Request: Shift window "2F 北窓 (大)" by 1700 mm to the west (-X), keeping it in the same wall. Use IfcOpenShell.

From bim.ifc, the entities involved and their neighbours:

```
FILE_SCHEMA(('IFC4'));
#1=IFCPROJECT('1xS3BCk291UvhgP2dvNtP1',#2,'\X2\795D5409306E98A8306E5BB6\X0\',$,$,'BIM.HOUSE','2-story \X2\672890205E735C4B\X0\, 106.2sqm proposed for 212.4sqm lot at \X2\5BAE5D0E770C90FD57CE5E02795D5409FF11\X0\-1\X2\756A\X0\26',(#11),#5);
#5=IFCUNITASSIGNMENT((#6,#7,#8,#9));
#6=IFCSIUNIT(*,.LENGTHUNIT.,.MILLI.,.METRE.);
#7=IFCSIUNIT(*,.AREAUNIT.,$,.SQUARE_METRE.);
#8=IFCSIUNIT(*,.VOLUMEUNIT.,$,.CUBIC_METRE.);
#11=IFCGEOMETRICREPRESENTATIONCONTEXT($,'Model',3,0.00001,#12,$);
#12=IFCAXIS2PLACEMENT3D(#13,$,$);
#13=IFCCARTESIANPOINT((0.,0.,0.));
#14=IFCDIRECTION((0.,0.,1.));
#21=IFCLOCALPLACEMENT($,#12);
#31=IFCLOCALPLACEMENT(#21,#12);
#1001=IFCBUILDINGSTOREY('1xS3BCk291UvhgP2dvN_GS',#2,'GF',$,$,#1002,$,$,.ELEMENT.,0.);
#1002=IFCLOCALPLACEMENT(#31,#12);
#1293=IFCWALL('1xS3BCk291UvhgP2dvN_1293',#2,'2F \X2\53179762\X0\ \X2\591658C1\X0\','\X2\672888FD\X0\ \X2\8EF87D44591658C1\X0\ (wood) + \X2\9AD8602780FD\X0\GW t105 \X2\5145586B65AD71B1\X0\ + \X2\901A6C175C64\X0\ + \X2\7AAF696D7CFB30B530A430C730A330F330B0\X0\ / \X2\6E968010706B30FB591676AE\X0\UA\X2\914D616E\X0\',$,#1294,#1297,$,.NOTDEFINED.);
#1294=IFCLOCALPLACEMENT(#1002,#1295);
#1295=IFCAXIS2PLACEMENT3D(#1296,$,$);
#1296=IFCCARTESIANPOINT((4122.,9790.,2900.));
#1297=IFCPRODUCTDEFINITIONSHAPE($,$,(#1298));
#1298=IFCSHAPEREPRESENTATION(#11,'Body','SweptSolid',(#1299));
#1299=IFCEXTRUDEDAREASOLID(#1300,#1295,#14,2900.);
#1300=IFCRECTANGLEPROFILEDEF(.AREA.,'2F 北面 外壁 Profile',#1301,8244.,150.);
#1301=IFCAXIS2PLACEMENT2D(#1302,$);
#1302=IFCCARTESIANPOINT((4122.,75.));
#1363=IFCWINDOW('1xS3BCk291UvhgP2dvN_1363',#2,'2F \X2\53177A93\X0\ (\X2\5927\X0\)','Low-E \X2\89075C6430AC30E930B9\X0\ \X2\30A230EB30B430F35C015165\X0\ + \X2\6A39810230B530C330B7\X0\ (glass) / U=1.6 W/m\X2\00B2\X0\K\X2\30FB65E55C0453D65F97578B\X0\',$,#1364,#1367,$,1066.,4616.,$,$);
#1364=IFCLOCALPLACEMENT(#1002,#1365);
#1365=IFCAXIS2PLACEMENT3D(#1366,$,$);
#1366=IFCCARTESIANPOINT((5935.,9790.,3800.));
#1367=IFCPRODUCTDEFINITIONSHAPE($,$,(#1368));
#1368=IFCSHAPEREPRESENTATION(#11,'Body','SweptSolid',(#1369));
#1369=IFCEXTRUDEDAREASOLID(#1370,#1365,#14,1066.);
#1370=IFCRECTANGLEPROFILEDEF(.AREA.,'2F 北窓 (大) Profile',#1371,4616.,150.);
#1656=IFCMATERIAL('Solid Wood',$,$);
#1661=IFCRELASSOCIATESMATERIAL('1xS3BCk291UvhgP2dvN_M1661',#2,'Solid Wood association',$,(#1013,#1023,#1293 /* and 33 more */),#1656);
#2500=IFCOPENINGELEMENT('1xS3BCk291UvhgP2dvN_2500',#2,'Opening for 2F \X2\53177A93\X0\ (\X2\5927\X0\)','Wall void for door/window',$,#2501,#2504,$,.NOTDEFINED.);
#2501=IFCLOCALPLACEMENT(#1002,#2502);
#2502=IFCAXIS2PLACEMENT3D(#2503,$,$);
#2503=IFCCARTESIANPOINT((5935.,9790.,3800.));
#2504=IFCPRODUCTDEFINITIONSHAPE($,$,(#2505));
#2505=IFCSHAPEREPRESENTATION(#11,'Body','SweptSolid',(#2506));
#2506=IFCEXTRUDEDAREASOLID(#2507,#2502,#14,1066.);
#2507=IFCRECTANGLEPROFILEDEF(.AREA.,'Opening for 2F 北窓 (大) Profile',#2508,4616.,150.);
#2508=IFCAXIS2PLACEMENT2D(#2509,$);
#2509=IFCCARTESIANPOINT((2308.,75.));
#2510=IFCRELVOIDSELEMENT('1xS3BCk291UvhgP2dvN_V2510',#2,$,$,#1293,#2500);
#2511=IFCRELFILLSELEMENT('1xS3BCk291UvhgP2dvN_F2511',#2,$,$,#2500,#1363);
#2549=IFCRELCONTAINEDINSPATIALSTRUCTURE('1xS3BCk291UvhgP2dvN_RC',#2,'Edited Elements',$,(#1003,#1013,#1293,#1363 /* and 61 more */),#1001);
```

```python
import ifcopenshell
import ifcopenshell.api.geometry
import ifcopenshell.util.placement
import ifcopenshell.util.unit

model = ifcopenshell.open("bim.ifc")
unit_scale = ifcopenshell.util.unit.calculate_unit_scale(model)

window = model.by_guid("1xS3BCk291UvhgP2dvN_1363")
opening = window.FillsVoids[0].RelatingOpeningElement
wall = opening.VoidsElements[0].RelatingBuildingElement

wall_matrix = ifcopenshell.util.placement.get_local_placement(wall.ObjectPlacement)
shift = wall_matrix[:3, 0] * -1.7 / unit_scale
before = ifcopenshell.util.placement.get_local_placement(window.ObjectPlacement)[:3, 3].copy()

# The window is not placed relative to its opening, so move both.
for product in (opening, window):
    matrix = ifcopenshell.util.placement.get_local_placement(product.ObjectPlacement)
    matrix[:3, 3] += shift
    ifcopenshell.api.geometry.edit_object_placement(model, product=product, matrix=matrix, is_si=False)

after = ifcopenshell.util.placement.get_local_placement(window.ObjectPlacement)[:3, 3]
print("window moved by", (after - before).round(3) + 0.0)

model.write("bim_rev.ifc")
```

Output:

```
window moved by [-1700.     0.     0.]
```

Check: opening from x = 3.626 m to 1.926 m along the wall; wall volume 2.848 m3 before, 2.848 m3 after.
